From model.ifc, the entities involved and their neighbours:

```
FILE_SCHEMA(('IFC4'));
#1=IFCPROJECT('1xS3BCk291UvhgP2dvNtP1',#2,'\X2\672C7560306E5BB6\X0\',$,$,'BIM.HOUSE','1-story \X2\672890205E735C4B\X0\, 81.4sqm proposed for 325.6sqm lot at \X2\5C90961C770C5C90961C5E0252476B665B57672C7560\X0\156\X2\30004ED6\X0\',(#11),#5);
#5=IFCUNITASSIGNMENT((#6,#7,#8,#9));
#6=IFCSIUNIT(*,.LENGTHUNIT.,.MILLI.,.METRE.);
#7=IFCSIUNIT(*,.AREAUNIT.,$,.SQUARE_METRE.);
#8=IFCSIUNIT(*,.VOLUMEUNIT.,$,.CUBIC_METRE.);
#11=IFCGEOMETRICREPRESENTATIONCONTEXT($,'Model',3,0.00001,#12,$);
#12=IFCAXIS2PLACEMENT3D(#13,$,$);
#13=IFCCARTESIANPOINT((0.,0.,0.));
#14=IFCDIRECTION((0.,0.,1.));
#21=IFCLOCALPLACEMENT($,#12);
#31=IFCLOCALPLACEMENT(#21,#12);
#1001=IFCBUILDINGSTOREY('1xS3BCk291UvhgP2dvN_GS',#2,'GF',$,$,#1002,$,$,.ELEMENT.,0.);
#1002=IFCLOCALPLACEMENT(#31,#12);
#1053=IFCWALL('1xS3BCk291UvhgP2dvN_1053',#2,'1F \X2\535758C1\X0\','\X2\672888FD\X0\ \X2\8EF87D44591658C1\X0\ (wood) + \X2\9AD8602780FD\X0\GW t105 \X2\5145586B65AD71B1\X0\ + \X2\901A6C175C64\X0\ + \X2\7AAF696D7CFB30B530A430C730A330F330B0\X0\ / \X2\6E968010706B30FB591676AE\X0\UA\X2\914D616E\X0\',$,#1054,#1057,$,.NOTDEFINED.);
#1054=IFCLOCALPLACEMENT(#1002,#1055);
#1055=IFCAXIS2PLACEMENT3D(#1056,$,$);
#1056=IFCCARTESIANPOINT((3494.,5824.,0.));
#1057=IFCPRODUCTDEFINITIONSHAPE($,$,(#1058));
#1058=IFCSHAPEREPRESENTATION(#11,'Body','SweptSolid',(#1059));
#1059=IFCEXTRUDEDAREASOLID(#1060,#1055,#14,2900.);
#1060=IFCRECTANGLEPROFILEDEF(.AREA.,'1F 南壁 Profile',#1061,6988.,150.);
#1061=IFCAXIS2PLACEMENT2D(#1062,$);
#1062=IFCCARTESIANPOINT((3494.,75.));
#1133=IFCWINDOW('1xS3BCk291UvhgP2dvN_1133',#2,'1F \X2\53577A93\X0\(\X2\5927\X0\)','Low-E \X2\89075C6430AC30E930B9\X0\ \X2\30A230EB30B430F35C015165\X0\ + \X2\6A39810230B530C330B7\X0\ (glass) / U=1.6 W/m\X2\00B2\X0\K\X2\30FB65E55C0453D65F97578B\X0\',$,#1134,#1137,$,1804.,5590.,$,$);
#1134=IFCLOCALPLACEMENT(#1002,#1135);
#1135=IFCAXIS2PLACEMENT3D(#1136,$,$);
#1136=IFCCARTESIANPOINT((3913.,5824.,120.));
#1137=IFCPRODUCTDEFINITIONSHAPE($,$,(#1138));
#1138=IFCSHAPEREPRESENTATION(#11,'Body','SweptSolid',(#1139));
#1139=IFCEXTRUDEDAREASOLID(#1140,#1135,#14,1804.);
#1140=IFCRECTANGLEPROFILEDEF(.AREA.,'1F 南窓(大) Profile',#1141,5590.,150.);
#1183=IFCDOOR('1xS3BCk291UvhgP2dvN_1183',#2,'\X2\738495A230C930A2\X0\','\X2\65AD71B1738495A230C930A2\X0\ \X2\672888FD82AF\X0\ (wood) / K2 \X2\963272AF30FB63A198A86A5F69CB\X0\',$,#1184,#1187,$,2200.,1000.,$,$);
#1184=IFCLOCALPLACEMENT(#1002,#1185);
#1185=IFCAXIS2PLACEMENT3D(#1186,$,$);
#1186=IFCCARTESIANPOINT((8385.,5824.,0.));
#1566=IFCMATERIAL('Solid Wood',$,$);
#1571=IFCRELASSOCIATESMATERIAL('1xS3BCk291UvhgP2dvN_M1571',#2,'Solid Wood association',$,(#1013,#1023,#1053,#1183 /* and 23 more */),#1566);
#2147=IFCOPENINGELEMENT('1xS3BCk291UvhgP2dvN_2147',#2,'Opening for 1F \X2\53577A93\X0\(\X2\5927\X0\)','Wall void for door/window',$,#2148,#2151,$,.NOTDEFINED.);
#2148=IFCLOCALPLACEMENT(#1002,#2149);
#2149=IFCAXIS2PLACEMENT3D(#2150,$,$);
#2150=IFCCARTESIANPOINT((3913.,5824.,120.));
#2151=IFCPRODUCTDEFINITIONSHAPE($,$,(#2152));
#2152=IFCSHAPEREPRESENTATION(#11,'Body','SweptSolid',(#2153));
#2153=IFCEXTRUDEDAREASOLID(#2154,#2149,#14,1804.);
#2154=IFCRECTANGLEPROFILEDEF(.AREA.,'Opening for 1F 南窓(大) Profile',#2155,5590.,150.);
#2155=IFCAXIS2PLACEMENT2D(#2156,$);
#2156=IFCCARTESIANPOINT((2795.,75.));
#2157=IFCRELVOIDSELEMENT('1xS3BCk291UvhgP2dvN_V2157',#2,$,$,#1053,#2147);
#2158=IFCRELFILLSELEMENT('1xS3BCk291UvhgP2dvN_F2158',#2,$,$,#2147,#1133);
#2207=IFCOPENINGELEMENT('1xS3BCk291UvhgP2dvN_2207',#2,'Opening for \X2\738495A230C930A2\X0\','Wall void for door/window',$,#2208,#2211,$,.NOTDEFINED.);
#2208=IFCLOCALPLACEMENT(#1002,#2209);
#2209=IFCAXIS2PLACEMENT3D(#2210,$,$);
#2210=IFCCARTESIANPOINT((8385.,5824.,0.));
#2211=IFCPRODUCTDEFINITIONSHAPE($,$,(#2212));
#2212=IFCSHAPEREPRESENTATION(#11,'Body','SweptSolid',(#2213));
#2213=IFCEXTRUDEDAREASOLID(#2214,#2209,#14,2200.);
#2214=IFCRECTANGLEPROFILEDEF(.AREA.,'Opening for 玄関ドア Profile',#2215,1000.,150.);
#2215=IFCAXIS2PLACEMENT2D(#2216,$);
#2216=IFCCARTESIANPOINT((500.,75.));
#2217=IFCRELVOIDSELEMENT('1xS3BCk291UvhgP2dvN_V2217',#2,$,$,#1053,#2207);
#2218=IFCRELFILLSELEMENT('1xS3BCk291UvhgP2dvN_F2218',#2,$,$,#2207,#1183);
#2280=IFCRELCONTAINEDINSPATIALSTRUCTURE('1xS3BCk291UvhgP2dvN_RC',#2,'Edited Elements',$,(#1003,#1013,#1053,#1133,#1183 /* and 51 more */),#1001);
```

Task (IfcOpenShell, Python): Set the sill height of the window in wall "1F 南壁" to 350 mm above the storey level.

```python
import numpy as np
import ifcopenshell
import ifcopenshell.api.geometry
import ifcopenshell.geom
import ifcopenshell.util.element
import ifcopenshell.util.placement
import ifcopenshell.util.shape
import ifcopenshell.util.unit

model = ifcopenshell.open("model.ifc")
unit_scale = ifcopenshell.util.unit.calculate_unit_scale(model)

window = model.by_guid("1xS3BCk291UvhgP2dvN_1133")
opening = window.FillsVoids[0].RelatingOpeningElement
storey = ifcopenshell.util.element.get_container(window, ifc_class="IfcBuildingStorey")
level = ifcopenshell.util.placement.get_local_placement(storey.ObjectPlacement)[2, 3]

# The opening's origin need not be at the sill, so measure its lowest point.
shape = ifcopenshell.geom.create_shape(ifcopenshell.geom.settings(), opening)
bottom = ifcopenshell.util.shape.get_shape_bottom_elevation(shape, shape.geometry) / unit_scale
dz = level + 0.35 / unit_scale - bottom

shift = np.array([0.0, 0.0, dz])
# The window is not placed relative to its opening, so move both.
for product in (opening, window):
    matrix = ifcopenshell.util.placement.get_local_placement(product.ObjectPlacement)
    matrix[:3, 3] += shift
    ifcopenshell.api.geometry.edit_object_placement(model, product=product, matrix=matrix, is_si=False)

print(f"moved by {dz * unit_scale:+.3f} m")

model.write("model_v2.ifc")
```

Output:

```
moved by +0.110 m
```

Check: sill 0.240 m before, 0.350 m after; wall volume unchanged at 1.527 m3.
